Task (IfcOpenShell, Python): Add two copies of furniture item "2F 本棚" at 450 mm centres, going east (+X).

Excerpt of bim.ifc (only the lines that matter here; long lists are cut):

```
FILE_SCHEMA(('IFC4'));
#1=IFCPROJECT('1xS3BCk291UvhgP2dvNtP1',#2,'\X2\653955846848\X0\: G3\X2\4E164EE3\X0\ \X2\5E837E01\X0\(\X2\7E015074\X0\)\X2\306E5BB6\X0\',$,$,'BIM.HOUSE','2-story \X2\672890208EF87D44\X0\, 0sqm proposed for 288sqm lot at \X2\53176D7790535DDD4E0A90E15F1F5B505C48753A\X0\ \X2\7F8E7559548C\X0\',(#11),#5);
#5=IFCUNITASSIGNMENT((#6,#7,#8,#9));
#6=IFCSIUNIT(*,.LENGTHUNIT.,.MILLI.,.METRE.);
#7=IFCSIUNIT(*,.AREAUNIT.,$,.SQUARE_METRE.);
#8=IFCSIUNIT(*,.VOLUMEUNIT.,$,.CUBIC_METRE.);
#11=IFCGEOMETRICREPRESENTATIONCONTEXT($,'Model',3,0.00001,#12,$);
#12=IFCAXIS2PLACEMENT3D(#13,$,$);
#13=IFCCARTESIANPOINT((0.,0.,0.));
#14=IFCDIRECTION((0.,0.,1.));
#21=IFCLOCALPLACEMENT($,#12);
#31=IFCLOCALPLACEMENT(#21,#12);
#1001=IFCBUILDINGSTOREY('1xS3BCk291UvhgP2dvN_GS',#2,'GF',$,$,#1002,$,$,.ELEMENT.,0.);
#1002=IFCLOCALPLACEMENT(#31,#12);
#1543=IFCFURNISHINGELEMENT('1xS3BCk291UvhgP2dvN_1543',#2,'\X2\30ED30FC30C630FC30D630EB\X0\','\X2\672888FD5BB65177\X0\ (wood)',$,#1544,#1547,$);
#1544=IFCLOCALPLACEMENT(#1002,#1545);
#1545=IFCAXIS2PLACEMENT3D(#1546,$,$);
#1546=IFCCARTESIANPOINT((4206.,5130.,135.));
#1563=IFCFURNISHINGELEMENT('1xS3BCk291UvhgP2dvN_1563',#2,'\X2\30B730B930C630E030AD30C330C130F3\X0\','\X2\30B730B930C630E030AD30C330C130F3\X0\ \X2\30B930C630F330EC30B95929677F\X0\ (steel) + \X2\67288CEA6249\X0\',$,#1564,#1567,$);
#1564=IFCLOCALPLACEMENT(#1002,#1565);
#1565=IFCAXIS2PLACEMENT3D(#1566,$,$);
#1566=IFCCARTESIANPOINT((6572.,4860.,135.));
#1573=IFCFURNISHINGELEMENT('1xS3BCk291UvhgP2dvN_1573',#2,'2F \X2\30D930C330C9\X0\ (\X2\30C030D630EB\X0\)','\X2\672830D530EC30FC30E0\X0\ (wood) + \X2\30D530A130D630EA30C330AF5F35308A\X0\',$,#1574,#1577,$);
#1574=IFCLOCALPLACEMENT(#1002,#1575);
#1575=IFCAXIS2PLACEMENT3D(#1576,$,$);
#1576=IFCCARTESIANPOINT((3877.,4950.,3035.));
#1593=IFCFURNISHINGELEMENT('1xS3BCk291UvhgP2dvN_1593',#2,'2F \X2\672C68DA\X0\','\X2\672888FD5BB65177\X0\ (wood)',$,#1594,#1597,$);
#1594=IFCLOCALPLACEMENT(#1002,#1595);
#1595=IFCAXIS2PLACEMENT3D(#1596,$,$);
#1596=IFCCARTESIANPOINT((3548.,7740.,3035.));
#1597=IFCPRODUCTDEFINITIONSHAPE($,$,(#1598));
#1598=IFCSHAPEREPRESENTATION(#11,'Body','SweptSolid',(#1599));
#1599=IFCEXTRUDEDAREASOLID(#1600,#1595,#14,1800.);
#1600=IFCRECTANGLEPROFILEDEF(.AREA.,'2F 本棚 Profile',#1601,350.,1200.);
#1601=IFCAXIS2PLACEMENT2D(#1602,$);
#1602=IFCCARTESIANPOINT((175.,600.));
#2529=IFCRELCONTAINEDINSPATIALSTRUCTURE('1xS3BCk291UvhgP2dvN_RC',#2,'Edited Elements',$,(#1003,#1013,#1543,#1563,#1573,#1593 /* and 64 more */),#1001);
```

```python
import numpy as np
import ifcopenshell
import ifcopenshell.api.geometry
import ifcopenshell.api.root
import ifcopenshell.util.element
import ifcopenshell.util.placement
import ifcopenshell.util.unit

model = ifcopenshell.open("bim.ifc")
unit_scale = ifcopenshell.util.unit.calculate_unit_scale(model)


def reuse_history(source, copy):
    """copy_class also copies each property set's owner history, people and application; keep the originals."""
    for rel in copy.IsDefinedBy:
        if rel.is_a("IfcRelDefinesByProperties") and (history := rel.RelatingPropertyDefinition.OwnerHistory):
            rel.RelatingPropertyDefinition.OwnerHistory = source.OwnerHistory
            ifcopenshell.util.element.remove_deep2(model, history)


source = model.by_id(1593)
base = ifcopenshell.util.placement.get_local_placement(source.ObjectPlacement)
step = np.array([1.0, 0.0, 0.0]) * 0.45 / unit_scale

for i in range(1, 3):
    copy = ifcopenshell.api.root.copy_class(model, product=source)
    copy.Representation = ifcopenshell.util.element.copy_deep(
        model, source.Representation, exclude=["IfcGeometricRepresentationContext", "IfcRepresentationMap"]
    )
    reuse_history(source, copy)
    matrix = base.copy()
    matrix[:3, 3] += i * step
    print("added at", matrix[:3, 3].round(3) + 0.0)
    ifcopenshell.api.geometry.edit_object_placement(model, product=copy, matrix=matrix, is_si=False)

model.write("bim_updated.ifc")
```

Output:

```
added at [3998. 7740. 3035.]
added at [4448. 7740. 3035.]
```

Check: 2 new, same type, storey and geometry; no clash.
